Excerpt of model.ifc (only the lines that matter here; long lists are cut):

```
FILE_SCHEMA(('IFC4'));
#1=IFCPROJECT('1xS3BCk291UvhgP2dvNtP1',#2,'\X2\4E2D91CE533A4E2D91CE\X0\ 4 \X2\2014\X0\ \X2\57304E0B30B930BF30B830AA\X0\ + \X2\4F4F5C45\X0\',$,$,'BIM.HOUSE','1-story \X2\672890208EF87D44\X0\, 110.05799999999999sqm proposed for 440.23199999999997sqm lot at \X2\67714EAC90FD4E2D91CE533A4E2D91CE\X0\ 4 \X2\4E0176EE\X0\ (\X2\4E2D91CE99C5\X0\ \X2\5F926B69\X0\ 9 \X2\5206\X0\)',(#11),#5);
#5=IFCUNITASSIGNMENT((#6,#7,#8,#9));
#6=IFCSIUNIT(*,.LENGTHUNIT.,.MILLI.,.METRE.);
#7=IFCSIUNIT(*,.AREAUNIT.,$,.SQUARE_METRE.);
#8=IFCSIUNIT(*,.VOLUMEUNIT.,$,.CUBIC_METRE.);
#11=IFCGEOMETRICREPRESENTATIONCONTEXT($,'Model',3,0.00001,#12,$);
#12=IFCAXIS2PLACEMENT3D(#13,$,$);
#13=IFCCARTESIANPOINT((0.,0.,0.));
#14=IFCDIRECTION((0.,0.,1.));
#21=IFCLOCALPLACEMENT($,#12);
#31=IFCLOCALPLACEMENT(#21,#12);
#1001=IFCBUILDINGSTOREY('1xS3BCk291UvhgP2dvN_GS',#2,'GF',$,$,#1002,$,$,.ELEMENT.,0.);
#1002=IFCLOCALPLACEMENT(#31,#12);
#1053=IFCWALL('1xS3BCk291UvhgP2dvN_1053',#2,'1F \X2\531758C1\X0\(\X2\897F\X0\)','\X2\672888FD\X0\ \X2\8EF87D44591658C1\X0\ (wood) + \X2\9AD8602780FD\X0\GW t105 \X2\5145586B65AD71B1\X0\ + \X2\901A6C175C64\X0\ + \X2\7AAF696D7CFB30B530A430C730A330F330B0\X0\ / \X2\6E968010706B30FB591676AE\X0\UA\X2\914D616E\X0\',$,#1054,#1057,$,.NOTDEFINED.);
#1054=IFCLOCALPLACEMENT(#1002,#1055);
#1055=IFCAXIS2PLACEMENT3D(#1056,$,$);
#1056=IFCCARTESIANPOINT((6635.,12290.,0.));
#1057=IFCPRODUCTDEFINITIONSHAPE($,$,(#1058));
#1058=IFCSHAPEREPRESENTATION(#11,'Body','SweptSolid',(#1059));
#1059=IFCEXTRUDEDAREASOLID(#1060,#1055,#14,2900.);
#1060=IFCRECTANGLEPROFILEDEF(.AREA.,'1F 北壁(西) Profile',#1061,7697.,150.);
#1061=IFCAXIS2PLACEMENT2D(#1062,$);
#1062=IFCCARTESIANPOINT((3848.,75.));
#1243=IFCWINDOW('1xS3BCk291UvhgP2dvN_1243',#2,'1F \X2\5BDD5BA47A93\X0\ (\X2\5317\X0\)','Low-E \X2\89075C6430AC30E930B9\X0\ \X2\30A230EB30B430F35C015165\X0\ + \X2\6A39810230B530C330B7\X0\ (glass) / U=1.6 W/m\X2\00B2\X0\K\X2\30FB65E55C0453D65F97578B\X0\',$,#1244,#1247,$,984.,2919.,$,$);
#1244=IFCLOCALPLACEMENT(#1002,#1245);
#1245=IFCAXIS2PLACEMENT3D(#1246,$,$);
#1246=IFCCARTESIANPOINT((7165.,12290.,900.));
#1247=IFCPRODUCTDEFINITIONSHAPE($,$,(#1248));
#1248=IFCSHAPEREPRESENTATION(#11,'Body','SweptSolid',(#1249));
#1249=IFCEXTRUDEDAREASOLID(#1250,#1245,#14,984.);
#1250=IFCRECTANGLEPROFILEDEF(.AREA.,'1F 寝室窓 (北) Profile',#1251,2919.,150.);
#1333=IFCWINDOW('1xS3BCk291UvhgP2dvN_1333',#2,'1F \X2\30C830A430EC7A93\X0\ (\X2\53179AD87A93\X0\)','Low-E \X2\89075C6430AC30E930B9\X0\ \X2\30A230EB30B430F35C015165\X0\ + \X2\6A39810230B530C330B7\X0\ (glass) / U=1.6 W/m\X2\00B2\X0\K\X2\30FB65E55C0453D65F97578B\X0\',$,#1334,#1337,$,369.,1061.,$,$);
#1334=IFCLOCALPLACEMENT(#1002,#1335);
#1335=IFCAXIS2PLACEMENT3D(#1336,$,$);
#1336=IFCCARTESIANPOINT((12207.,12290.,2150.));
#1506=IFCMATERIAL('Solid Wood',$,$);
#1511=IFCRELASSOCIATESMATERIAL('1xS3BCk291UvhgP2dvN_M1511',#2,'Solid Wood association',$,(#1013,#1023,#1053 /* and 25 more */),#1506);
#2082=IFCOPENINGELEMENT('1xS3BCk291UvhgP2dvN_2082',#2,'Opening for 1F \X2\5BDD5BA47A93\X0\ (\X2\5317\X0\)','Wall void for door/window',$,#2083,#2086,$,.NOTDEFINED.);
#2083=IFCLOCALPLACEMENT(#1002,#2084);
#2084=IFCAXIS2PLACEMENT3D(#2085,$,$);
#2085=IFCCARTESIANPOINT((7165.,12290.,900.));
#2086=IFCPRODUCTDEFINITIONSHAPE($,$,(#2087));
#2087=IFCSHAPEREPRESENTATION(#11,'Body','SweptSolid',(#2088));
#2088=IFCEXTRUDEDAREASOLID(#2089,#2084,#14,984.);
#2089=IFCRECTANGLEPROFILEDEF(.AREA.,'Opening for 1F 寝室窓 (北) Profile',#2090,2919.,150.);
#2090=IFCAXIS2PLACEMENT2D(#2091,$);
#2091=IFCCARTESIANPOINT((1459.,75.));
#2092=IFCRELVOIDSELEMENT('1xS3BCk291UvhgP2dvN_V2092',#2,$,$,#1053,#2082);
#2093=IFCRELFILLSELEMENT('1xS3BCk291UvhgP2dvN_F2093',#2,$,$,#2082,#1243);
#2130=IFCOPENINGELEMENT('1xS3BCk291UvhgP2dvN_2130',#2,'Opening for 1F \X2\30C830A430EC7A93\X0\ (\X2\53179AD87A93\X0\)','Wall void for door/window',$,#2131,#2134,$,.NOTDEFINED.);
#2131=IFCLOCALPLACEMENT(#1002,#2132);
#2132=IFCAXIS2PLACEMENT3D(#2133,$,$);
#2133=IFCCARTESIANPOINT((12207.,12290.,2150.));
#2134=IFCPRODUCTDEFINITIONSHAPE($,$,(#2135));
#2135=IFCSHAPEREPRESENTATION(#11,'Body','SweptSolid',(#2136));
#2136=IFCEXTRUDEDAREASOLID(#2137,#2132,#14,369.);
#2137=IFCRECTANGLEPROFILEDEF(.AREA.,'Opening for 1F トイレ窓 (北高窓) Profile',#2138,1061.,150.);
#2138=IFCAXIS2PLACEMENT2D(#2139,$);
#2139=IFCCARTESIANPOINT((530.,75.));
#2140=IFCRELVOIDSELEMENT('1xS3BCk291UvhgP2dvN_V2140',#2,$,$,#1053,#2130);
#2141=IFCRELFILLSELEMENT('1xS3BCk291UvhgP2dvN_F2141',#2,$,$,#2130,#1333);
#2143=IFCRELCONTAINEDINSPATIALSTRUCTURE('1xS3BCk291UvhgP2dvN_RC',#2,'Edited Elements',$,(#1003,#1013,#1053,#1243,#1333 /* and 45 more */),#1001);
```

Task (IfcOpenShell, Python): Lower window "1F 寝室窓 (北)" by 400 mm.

```python
import numpy as np
import ifcopenshell
import ifcopenshell.api.geometry
import ifcopenshell.util.placement
import ifcopenshell.util.unit

model = ifcopenshell.open("model.ifc")
unit_scale = ifcopenshell.util.unit.calculate_unit_scale(model)

window = model.by_guid("1xS3BCk291UvhgP2dvN_1243")
opening = window.FillsVoids[0].RelatingOpeningElement
dz = -0.4 / unit_scale

shift = np.array([0.0, 0.0, dz])
# The window is not placed relative to its opening, so move both.
for product in (opening, window):
    matrix = ifcopenshell.util.placement.get_local_placement(product.ObjectPlacement)
    matrix[:3, 3] += shift
    ifcopenshell.api.geometry.edit_object_placement(model, product=product, matrix=matrix, is_si=False)

print(f"moved by {dz * unit_scale:+.3f} m")

model.write("model-out.ifc")
```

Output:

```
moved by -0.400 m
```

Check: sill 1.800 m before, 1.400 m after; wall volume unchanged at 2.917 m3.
